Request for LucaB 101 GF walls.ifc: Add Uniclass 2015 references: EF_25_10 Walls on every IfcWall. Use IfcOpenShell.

First a look at what the model holds.

```python
import ifcopenshell

model = ifcopenshell.open("LucaB 101 GF walls.ifc")
print(model.schema)
print("classifications:", [c.Name for c in model.by_type("IfcClassification")])
for ifc_class in ("IfcDoor", "IfcRoof", "IfcStair", "IfcWall", "IfcWindow"):
    print(ifc_class, len(model.by_type(ifc_class)))
```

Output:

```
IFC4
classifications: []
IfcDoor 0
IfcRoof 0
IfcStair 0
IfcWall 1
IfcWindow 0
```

```python
import ifcopenshell
import ifcopenshell.api.classification

model = ifcopenshell.open("LucaB 101 GF walls.ifc")

system = ifcopenshell.api.classification.add_classification(model, classification="Uniclass 2015")

codes = {
    "IfcWall": ("EF_25_10", "Walls"),
}
for ifc_class, (code, name) in codes.items():
    products = model.by_type(ifc_class)
    ifcopenshell.api.classification.add_reference(
        model, products=products, classification=system, identification=code, name=name
    )
    print(code, len(products))

model.write("LucaB 101 GF walls_updated.ifc")
```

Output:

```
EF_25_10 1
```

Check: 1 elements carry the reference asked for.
